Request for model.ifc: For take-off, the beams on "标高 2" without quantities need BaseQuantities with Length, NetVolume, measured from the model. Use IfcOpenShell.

First a look at what the model holds.

```python
import ifcopenshell
import ifcopenshell.util.element
import ifcopenshell.util.unit

model = ifcopenshell.open("model.ifc")
print(model.schema)
for unit_type in ("LENGTHUNIT", "AREAUNIT", "VOLUMEUNIT"):
    print(unit_type, ifcopenshell.util.unit.calculate_unit_scale(model, unit_type))
storey = next(s for s in model.by_type("IfcBuildingStorey") if s.Name == "标高 2")
beams = [e for e in ifcopenshell.util.element.get_decomposition(storey) if e.is_a("IfcBeam")]
for e in sorted(beams, key=lambda e: e.id()):
    print(e.id(), e.is_a(), e.Name, list(ifcopenshell.util.element.get_psets(e, qtos_only=True)), sep=" | ")
```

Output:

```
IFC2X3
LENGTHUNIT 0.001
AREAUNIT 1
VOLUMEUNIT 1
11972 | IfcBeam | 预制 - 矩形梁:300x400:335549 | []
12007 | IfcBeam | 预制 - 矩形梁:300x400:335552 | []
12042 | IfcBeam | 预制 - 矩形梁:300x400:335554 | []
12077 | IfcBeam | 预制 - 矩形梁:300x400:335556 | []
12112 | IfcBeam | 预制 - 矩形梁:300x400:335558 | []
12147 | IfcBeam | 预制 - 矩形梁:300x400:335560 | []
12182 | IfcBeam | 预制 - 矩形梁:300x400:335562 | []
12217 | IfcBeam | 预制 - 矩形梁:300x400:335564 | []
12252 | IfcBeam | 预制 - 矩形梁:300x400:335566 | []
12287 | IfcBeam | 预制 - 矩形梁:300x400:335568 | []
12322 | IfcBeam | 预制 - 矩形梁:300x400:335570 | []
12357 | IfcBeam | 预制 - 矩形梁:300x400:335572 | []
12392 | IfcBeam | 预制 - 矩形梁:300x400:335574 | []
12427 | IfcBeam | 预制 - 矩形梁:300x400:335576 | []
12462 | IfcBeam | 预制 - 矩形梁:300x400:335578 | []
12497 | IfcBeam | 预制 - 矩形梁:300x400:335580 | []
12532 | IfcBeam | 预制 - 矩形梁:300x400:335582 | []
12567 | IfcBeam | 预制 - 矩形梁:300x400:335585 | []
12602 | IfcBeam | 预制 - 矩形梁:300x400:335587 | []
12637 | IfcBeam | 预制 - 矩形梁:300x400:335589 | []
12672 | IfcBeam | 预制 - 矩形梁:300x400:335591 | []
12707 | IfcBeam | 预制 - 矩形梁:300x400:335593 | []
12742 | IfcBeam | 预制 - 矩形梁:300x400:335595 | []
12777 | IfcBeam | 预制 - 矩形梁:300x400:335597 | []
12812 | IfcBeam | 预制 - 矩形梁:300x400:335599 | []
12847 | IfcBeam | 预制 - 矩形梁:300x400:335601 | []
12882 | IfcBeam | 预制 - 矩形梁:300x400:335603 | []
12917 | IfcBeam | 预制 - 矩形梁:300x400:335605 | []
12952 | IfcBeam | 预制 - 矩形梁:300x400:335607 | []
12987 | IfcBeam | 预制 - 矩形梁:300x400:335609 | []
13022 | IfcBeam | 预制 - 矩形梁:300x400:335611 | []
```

```python
import ifcopenshell
import ifcopenshell.api.pset
import ifcopenshell.geom
import ifcopenshell.util.element
import ifcopenshell.util.shape
import ifcopenshell.util.unit

model = ifcopenshell.open("model.ifc")
unit_scale = ifcopenshell.util.unit.calculate_unit_scale(model)
volume_scale = ifcopenshell.util.unit.calculate_unit_scale(model, "VOLUMEUNIT")
settings = ifcopenshell.geom.settings()

storey = next(s for s in model.by_type("IfcBuildingStorey") if s.Name == "标高 2")
beams = [e for e in ifcopenshell.util.element.get_decomposition(storey) if e.is_a("IfcBeam")]

for e in sorted(beams, key=lambda e: e.id()):
    if ifcopenshell.util.element.get_psets(e, qtos_only=True, should_inherit=False):
        continue
    # Geometry comes back in metres, in the element's own axes.
    shape = ifcopenshell.geom.create_shape(settings, e)
    values = {
        "Length": ifcopenshell.util.shape.get_max_xyz(shape.geometry) / unit_scale,
        "NetVolume": ifcopenshell.util.shape.get_volume(shape.geometry) / volume_scale,
    }
    qto = ifcopenshell.api.pset.add_qto(model, product=e, name="BaseQuantities")
    ifcopenshell.api.pset.edit_qto(model, qto=qto, properties=values)
    print(e.id(), {k: round(v, 3) for k, v in values.items()})

model.write("model_edited.ifc")
```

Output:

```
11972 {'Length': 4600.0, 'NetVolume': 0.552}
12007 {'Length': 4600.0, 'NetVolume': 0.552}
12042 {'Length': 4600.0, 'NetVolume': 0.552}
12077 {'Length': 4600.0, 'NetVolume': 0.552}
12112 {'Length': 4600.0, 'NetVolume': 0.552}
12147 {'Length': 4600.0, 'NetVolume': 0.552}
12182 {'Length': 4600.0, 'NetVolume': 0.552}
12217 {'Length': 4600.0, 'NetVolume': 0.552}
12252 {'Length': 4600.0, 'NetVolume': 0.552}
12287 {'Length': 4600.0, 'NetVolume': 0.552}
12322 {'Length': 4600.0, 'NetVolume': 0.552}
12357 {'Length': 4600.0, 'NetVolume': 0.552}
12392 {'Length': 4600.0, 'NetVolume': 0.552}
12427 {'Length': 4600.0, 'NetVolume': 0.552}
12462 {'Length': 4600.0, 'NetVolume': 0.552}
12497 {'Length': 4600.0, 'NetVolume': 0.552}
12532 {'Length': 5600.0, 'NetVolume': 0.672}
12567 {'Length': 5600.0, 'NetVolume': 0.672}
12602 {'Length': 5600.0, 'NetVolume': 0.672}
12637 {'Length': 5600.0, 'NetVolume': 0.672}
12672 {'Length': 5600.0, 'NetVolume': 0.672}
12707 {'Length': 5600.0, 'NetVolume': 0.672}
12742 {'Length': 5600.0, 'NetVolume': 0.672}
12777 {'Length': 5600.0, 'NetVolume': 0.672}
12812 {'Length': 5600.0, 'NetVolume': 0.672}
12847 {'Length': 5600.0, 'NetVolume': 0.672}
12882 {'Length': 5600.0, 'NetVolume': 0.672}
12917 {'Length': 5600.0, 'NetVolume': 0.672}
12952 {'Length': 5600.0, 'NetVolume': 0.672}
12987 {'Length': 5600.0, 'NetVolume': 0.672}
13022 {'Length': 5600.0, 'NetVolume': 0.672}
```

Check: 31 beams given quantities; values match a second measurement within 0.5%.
